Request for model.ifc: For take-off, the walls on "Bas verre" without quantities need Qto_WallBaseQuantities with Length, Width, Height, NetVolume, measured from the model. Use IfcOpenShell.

First a look at what the model holds.

```python
import ifcopenshell
import ifcopenshell.util.element
import ifcopenshell.util.unit

model = ifcopenshell.open("model.ifc")
print(model.schema)
for unit_type in ("LENGTHUNIT", "AREAUNIT", "VOLUMEUNIT"):
    print(unit_type, ifcopenshell.util.unit.calculate_unit_scale(model, unit_type))
storey = next(s for s in model.by_type("IfcBuildingStorey") if s.Name == "Bas verre")
walls = [e for e in ifcopenshell.util.element.get_decomposition(storey) if e.is_a("IfcWall")]
for e in sorted(walls, key=lambda e: e.id()):
    print(e.id(), e.is_a(), e.Name, list(ifcopenshell.util.element.get_psets(e, qtos_only=True)), sep=" | ")
```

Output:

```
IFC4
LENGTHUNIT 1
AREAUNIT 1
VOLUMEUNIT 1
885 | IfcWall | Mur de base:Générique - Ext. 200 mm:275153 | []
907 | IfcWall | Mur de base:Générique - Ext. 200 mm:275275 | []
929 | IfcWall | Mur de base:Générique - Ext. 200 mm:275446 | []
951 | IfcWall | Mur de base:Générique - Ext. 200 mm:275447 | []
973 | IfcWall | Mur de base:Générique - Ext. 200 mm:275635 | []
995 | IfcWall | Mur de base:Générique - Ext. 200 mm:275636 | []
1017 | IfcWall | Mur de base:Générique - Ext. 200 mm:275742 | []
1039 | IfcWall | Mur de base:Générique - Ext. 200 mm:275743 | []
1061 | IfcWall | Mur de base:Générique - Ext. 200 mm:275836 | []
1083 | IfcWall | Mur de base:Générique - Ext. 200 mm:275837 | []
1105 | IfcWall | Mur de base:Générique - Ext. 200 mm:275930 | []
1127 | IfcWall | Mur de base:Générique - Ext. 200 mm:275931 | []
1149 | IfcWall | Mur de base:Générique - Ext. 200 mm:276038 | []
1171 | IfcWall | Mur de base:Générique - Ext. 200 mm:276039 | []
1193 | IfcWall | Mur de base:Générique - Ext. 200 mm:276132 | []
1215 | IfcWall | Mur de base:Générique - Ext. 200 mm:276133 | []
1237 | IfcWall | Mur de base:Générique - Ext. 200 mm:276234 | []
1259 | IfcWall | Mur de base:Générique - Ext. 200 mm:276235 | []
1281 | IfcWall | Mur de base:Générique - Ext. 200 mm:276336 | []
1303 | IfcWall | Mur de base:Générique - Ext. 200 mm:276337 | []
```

```python
import ifcopenshell
import ifcopenshell.api.pset
import ifcopenshell.geom
import ifcopenshell.util.element
import ifcopenshell.util.shape
import ifcopenshell.util.unit

model = ifcopenshell.open("model.ifc")
unit_scale = ifcopenshell.util.unit.calculate_unit_scale(model)
volume_scale = ifcopenshell.util.unit.calculate_unit_scale(model, "VOLUMEUNIT")
settings = ifcopenshell.geom.settings()

storey = next(s for s in model.by_type("IfcBuildingStorey") if s.Name == "Bas verre")
walls = [e for e in ifcopenshell.util.element.get_decomposition(storey) if e.is_a("IfcWall")]

for e in sorted(walls, key=lambda e: e.id()):
    if ifcopenshell.util.element.get_psets(e, qtos_only=True, should_inherit=False):
        continue
    # Geometry comes back in metres, in the element's own axes.
    shape = ifcopenshell.geom.create_shape(settings, e)
    values = {
        "Length": ifcopenshell.util.shape.get_x(shape.geometry) / unit_scale,
        "Width": ifcopenshell.util.shape.get_y(shape.geometry) / unit_scale,
        "Height": ifcopenshell.util.shape.get_z(shape.geometry) / unit_scale,
        "NetVolume": ifcopenshell.util.shape.get_volume(shape.geometry) / volume_scale,
    }
    qto = ifcopenshell.api.pset.add_qto(model, product=e, name="Qto_WallBaseQuantities")
    ifcopenshell.api.pset.edit_qto(model, qto=qto, properties=values)
    print(e.id(), {k: round(v, 3) for k, v in values.items()})

model.write("model-out.ifc")
```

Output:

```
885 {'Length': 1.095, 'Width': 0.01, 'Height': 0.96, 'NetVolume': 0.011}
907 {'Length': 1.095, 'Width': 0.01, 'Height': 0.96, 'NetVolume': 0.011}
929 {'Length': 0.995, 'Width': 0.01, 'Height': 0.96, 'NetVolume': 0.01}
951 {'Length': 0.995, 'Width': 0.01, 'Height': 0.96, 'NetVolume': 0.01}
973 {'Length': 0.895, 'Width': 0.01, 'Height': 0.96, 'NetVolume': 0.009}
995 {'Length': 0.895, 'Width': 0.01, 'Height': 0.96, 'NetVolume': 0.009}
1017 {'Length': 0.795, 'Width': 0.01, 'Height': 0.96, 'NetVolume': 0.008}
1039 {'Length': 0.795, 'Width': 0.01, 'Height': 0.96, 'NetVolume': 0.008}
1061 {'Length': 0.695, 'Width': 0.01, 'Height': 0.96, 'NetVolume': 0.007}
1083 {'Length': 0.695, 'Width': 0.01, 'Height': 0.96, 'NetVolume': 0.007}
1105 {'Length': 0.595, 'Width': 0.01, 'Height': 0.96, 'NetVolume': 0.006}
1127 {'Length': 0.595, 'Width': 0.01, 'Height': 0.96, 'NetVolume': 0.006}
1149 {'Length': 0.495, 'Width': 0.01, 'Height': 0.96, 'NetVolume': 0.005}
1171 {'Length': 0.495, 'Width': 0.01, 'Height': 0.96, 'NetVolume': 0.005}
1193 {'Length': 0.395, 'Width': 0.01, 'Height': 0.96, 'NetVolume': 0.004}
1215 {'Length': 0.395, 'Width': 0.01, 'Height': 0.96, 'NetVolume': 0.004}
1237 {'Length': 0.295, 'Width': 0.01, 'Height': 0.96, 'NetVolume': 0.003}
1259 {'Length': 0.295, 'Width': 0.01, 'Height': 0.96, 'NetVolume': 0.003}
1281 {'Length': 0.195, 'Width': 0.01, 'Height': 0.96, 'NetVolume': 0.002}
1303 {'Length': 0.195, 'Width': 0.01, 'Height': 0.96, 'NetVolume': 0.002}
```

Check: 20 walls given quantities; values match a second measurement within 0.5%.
